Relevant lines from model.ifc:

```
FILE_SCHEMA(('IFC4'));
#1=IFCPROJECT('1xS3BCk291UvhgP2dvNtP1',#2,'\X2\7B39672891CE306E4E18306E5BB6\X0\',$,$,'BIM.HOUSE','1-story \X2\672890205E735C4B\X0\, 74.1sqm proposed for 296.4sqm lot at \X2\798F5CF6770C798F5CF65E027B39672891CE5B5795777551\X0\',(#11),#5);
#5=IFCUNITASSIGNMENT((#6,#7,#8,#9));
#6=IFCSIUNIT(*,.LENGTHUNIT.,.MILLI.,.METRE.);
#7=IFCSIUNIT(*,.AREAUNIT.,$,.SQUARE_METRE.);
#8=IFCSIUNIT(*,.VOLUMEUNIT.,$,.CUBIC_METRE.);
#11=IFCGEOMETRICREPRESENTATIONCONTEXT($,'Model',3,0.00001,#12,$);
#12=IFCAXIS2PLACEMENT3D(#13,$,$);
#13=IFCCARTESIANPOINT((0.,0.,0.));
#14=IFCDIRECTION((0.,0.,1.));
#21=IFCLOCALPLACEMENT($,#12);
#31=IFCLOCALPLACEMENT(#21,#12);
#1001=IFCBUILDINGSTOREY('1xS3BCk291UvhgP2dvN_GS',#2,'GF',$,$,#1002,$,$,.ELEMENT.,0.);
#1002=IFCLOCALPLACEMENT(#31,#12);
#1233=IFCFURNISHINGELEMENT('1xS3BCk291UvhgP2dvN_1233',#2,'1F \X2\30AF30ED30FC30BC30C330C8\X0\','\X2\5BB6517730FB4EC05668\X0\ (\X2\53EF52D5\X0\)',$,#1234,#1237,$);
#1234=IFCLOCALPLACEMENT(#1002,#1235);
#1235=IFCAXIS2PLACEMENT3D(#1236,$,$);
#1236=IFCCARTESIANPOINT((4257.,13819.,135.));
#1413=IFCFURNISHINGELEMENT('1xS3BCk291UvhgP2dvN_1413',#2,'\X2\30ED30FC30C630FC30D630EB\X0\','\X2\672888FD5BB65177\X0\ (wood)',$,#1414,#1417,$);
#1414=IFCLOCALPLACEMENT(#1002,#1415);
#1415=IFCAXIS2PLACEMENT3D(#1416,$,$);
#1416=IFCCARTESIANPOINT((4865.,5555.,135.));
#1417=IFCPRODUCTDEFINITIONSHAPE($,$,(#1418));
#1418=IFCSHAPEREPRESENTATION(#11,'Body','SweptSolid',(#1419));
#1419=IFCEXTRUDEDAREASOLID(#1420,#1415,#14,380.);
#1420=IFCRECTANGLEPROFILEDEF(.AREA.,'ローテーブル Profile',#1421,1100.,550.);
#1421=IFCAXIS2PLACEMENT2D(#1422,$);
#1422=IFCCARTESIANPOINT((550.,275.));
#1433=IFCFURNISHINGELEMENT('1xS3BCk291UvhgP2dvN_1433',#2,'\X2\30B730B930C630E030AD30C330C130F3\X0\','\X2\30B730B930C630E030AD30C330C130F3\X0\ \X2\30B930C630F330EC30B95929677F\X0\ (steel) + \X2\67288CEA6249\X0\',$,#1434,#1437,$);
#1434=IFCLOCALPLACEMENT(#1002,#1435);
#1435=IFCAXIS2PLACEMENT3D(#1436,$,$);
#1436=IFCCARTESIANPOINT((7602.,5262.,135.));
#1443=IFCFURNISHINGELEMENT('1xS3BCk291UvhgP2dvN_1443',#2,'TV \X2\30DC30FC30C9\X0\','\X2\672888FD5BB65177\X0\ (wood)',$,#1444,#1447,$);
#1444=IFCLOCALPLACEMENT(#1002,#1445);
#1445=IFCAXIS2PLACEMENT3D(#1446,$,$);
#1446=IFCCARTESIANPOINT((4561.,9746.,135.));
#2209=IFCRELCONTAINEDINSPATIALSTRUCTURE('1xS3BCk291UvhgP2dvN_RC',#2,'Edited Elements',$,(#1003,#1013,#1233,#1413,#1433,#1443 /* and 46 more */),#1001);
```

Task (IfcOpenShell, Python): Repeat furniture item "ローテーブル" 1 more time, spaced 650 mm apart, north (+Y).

```python
import numpy as np
import ifcopenshell
import ifcopenshell.api.geometry
import ifcopenshell.api.root
import ifcopenshell.util.element
import ifcopenshell.util.placement
import ifcopenshell.util.unit

model = ifcopenshell.open("model.ifc")
unit_scale = ifcopenshell.util.unit.calculate_unit_scale(model)


def reuse_history(source, copy):
    """copy_class also copies each property set's owner history, people and application; keep the originals."""
    for rel in copy.IsDefinedBy:
        if rel.is_a("IfcRelDefinesByProperties") and (history := rel.RelatingPropertyDefinition.OwnerHistory):
            rel.RelatingPropertyDefinition.OwnerHistory = source.OwnerHistory
            ifcopenshell.util.element.remove_deep2(model, history)


source = model.by_guid("1xS3BCk291UvhgP2dvN_1413")
base = ifcopenshell.util.placement.get_local_placement(source.ObjectPlacement)
step = np.array([0.0, 1.0, 0.0]) * 0.65 / unit_scale

for i in range(1, 2):
    copy = ifcopenshell.api.root.copy_class(model, product=source)
    copy.Representation = ifcopenshell.util.element.copy_deep(
        model, source.Representation, exclude=["IfcGeometricRepresentationContext", "IfcRepresentationMap"]
    )
    reuse_history(source, copy)
    matrix = base.copy()
    matrix[:3, 3] += i * step
    print("added at", matrix[:3, 3].round(3) + 0.0)
    ifcopenshell.api.geometry.edit_object_placement(model, product=copy, matrix=matrix, is_si=False)

model.write("model-out.ifc")
```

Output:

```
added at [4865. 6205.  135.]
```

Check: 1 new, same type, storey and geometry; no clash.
